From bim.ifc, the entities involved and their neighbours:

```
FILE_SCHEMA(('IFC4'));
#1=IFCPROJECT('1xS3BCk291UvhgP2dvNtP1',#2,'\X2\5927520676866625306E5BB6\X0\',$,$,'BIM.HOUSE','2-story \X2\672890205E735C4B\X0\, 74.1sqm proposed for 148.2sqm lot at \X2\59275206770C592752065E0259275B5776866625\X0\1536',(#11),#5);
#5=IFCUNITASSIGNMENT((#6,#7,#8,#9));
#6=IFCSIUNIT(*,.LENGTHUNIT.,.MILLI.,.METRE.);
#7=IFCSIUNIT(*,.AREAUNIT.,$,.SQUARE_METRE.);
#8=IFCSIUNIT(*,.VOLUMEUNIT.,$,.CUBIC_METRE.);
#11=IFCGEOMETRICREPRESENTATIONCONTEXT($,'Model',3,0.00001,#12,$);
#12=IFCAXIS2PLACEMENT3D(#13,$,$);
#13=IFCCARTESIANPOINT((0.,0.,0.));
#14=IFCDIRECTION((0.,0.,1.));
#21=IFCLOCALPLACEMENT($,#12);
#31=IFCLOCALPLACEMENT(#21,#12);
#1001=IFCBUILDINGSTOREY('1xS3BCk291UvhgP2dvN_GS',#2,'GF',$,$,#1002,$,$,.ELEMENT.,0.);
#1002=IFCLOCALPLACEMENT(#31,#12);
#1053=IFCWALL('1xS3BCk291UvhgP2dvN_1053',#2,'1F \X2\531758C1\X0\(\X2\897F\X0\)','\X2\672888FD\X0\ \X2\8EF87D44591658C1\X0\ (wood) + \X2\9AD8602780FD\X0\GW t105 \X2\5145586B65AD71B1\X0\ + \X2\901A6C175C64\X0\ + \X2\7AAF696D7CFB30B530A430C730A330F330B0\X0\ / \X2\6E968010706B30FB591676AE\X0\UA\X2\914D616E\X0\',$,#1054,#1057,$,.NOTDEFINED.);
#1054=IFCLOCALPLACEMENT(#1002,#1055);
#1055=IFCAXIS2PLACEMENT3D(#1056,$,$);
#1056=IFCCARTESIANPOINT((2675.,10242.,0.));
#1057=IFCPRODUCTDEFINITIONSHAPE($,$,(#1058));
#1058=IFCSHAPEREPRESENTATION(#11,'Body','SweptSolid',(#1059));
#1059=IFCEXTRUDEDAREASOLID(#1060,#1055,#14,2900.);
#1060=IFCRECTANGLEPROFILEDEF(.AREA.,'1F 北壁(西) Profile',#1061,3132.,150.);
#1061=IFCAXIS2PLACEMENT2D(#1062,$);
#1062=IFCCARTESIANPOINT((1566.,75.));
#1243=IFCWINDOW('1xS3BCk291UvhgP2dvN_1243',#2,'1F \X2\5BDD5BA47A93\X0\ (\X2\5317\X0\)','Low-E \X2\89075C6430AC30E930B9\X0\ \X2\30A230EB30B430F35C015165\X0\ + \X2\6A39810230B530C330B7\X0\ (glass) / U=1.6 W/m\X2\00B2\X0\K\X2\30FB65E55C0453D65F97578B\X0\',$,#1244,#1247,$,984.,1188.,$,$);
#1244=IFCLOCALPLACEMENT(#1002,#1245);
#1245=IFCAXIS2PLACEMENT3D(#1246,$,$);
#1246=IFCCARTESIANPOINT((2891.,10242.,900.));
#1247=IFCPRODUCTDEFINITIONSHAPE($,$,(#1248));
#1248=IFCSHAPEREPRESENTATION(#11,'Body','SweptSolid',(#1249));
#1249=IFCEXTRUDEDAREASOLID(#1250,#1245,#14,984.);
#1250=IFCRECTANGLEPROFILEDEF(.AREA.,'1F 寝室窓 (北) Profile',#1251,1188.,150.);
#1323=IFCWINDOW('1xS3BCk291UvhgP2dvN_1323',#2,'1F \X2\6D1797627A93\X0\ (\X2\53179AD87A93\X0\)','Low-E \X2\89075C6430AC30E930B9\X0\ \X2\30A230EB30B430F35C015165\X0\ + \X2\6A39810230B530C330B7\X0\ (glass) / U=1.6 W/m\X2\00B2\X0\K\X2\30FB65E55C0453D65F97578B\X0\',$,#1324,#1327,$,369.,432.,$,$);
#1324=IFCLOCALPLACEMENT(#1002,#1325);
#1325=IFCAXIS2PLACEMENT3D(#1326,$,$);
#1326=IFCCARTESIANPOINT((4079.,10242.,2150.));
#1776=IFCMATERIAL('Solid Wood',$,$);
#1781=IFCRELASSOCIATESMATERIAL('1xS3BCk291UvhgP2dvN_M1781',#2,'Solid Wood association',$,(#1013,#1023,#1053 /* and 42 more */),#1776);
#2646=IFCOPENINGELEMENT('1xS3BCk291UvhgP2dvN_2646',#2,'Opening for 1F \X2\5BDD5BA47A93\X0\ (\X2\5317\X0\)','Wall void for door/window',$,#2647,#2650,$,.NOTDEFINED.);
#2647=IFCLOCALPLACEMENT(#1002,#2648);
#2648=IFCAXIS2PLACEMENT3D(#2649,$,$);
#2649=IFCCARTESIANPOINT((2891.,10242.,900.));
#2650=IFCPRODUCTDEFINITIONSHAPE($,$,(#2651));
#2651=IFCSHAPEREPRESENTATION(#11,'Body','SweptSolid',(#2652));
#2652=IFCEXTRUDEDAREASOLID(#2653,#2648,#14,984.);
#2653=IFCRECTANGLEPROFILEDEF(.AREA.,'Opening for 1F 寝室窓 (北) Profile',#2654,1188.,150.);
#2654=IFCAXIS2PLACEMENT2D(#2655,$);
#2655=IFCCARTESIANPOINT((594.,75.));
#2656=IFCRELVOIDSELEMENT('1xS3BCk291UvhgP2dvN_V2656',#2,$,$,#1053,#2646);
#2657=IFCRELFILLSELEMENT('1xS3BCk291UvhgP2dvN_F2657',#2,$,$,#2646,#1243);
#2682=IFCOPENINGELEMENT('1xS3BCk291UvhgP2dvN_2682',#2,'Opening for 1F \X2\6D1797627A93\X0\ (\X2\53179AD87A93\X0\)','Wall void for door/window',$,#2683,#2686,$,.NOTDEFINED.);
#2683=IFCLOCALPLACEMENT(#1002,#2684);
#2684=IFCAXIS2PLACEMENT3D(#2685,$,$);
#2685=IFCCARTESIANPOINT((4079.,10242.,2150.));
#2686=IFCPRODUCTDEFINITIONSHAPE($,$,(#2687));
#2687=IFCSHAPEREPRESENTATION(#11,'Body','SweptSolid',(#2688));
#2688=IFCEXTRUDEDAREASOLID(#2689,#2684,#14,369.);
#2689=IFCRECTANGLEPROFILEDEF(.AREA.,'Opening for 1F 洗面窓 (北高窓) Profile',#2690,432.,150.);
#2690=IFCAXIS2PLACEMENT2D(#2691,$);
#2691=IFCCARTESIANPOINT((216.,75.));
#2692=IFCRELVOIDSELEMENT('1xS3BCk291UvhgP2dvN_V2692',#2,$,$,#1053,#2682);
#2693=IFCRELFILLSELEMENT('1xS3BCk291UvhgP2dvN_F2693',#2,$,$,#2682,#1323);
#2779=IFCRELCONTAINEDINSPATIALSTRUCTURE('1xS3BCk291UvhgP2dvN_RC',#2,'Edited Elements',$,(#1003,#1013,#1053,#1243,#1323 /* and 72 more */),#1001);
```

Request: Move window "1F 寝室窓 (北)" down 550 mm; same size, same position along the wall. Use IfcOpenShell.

```python
import numpy as np
import ifcopenshell
import ifcopenshell.api.geometry
import ifcopenshell.util.placement
import ifcopenshell.util.unit

model = ifcopenshell.open("bim.ifc")
unit_scale = ifcopenshell.util.unit.calculate_unit_scale(model)

window = model.by_guid("1xS3BCk291UvhgP2dvN_1243")
opening = window.FillsVoids[0].RelatingOpeningElement
dz = -550.0

shift = np.array([0.0, 0.0, dz])
# The window is not placed relative to its opening, so move both.
for product in (opening, window):
    matrix = ifcopenshell.util.placement.get_local_placement(product.ObjectPlacement)
    matrix[:3, 3] += shift
    ifcopenshell.api.geometry.edit_object_placement(model, product=product, matrix=matrix, is_si=False)

print(f"moved by {dz * unit_scale:+.3f} m")

model.write("bim_rev.ifc")
```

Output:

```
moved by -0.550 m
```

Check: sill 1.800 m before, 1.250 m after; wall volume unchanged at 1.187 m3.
